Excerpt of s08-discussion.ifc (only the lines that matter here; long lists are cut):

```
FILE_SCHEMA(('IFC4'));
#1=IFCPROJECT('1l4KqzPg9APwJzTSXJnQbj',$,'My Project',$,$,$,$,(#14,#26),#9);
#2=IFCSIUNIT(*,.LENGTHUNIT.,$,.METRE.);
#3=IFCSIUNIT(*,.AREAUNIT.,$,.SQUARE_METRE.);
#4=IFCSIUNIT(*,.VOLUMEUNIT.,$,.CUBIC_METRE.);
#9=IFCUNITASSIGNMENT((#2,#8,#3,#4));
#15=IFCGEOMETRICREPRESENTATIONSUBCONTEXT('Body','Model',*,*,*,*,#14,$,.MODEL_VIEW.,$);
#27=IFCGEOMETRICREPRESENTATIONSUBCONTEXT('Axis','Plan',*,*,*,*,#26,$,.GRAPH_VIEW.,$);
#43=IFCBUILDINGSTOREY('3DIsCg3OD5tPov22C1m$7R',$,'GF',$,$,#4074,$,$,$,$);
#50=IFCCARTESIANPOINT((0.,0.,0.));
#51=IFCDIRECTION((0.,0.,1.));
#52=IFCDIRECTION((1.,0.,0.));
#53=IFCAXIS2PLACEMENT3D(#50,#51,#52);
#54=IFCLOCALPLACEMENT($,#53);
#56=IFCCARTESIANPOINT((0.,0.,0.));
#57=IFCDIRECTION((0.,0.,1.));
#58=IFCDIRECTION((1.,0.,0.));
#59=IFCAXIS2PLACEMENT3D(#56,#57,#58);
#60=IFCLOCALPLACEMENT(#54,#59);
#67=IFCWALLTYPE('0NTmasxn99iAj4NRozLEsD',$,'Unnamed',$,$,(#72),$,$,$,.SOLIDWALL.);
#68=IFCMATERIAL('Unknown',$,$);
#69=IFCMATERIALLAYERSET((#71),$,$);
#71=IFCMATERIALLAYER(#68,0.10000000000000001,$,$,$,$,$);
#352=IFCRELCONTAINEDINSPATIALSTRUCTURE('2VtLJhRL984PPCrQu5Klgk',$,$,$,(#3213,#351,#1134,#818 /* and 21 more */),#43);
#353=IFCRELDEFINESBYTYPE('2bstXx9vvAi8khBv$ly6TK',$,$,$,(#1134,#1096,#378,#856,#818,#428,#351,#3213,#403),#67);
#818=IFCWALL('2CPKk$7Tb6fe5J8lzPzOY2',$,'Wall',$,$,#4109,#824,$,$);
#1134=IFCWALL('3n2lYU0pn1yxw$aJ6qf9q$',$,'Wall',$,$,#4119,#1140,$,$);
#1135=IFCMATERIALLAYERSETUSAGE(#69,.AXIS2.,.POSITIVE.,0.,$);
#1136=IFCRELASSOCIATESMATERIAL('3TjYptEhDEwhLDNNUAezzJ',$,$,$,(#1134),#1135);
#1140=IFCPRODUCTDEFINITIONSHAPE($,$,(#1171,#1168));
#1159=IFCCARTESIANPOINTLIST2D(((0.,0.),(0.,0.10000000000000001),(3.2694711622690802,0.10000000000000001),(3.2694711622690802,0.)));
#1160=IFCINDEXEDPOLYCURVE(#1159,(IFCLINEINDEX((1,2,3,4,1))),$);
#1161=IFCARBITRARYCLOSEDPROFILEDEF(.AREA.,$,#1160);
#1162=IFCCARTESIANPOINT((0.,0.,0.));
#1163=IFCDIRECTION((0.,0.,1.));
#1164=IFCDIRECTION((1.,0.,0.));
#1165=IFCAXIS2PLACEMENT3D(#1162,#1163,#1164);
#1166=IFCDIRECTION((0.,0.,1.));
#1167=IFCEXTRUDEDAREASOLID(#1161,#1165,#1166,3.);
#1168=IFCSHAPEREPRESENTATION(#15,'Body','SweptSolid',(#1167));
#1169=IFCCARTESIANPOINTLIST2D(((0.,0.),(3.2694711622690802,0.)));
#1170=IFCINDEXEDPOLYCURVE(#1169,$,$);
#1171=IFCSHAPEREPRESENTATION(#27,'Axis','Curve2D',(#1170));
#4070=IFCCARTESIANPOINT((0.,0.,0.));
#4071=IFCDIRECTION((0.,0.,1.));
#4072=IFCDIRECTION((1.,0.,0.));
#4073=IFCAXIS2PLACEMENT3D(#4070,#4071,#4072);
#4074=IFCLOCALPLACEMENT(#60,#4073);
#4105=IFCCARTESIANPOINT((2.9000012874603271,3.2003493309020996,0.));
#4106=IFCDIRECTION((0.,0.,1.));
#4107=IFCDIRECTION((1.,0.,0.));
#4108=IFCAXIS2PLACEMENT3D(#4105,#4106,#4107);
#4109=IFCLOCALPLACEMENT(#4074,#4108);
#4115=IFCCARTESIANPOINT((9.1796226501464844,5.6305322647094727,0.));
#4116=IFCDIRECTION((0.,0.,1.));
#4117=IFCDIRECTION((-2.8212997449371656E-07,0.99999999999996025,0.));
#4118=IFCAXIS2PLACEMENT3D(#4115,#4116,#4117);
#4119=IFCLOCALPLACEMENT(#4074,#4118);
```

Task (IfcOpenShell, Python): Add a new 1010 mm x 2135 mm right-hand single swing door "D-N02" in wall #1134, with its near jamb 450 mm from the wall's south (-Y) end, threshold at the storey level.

```python
import numpy as np
import ifcopenshell
import ifcopenshell.api.feature
import ifcopenshell.api.geometry
import ifcopenshell.api.root
import ifcopenshell.api.spatial
import ifcopenshell.geom
import ifcopenshell.util.element
import ifcopenshell.util.placement
import ifcopenshell.util.representation
import ifcopenshell.util.shape
import ifcopenshell.util.unit

model = ifcopenshell.open("s08-discussion.ifc")
unit_scale = ifcopenshell.util.unit.calculate_unit_scale(model)
settings = ifcopenshell.geom.settings()


def volume(element):
    """Net volume in cubic metres, openings subtracted."""
    shape = ifcopenshell.geom.create_shape(settings, element)
    return ifcopenshell.util.shape.get_volume(shape.geometry)


wall = model.by_id(1134)
storey = ifcopenshell.util.element.get_container(wall, ifc_class="IfcBuildingStorey")
context = ifcopenshell.util.representation.get_context(model, "Model", "Body", "MODEL_VIEW")
before = volume(wall)

width, height, from_end, sill = 1.01, 2.135, 0.45, 0.0  # metres

# The wall runs along its own X axis, and the end named is its -X end.
wall_shape = ifcopenshell.geom.create_shape(settings, wall)
x, y, z = ifcopenshell.util.shape.get_vertices(wall_shape.geometry).T
start = x.min() + from_end
face, thickness = float(y.min()), float(y.max() - y.min())
wall_matrix = ifcopenshell.util.placement.get_local_placement(wall.ObjectPlacement)
level = ifcopenshell.util.placement.get_local_placement(storey.ObjectPlacement)[2, 3]


def in_wall(x, y):
    """Placement at x, y metres in the wall's axes, at sill height."""
    matrix = wall_matrix.copy()
    matrix[:, 3] = wall_matrix @ np.array([x / unit_scale, y / unit_scale, 0.0, 1.0])
    matrix[2, 3] = level + sill / unit_scale
    return matrix


# Opening: a box that overshoots both wall faces by 50 mm.
opening = ifcopenshell.api.root.create_entity(model, ifc_class="IfcOpeningElement", predefined_type="OPENING")
box = ifcopenshell.api.geometry.add_wall_representation(
    model, context=context, length=width, height=height, thickness=thickness + 0.1
)
ifcopenshell.api.geometry.assign_representation(model, product=opening, representation=box)
ifcopenshell.api.geometry.edit_object_placement(model, product=opening, matrix=in_wall(start, face - 0.05), is_si=False)
ifcopenshell.api.feature.add_feature(model, feature=opening, element=wall)

door = ifcopenshell.api.root.create_entity(model, ifc_class="IfcDoor", name="D-N02", predefined_type="DOOR")
door.OverallWidth, door.OverallHeight = width / unit_scale, height / unit_scale
door.OperationType = "SINGLE_SWING_RIGHT"
body = ifcopenshell.api.geometry.add_door_representation(
    model,
    context=context,
    overall_width=door.OverallWidth,
    overall_height=door.OverallHeight,
    operation_type="SINGLE_SWING_RIGHT",
    lining_properties={"LiningDepth": thickness / unit_scale, "ThresholdDepth": thickness / unit_scale},
)
ifcopenshell.api.geometry.assign_representation(model, product=door, representation=body)
ifcopenshell.api.spatial.assign_container(model, products=[door], relating_structure=storey)
ifcopenshell.api.feature.add_filling(model, opening=opening, element=door)

# The lining spans the wall, so the door starts at the wall face.
ifcopenshell.api.geometry.edit_object_placement(model, product=door, matrix=in_wall(start, face), is_si=False)

after = volume(wall)

print(f"wall volume {before:.3f} -> {after:.3f} m3")

model.write("s08-discussion_edited.ifc")
```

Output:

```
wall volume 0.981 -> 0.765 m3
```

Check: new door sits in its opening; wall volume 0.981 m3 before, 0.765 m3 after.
